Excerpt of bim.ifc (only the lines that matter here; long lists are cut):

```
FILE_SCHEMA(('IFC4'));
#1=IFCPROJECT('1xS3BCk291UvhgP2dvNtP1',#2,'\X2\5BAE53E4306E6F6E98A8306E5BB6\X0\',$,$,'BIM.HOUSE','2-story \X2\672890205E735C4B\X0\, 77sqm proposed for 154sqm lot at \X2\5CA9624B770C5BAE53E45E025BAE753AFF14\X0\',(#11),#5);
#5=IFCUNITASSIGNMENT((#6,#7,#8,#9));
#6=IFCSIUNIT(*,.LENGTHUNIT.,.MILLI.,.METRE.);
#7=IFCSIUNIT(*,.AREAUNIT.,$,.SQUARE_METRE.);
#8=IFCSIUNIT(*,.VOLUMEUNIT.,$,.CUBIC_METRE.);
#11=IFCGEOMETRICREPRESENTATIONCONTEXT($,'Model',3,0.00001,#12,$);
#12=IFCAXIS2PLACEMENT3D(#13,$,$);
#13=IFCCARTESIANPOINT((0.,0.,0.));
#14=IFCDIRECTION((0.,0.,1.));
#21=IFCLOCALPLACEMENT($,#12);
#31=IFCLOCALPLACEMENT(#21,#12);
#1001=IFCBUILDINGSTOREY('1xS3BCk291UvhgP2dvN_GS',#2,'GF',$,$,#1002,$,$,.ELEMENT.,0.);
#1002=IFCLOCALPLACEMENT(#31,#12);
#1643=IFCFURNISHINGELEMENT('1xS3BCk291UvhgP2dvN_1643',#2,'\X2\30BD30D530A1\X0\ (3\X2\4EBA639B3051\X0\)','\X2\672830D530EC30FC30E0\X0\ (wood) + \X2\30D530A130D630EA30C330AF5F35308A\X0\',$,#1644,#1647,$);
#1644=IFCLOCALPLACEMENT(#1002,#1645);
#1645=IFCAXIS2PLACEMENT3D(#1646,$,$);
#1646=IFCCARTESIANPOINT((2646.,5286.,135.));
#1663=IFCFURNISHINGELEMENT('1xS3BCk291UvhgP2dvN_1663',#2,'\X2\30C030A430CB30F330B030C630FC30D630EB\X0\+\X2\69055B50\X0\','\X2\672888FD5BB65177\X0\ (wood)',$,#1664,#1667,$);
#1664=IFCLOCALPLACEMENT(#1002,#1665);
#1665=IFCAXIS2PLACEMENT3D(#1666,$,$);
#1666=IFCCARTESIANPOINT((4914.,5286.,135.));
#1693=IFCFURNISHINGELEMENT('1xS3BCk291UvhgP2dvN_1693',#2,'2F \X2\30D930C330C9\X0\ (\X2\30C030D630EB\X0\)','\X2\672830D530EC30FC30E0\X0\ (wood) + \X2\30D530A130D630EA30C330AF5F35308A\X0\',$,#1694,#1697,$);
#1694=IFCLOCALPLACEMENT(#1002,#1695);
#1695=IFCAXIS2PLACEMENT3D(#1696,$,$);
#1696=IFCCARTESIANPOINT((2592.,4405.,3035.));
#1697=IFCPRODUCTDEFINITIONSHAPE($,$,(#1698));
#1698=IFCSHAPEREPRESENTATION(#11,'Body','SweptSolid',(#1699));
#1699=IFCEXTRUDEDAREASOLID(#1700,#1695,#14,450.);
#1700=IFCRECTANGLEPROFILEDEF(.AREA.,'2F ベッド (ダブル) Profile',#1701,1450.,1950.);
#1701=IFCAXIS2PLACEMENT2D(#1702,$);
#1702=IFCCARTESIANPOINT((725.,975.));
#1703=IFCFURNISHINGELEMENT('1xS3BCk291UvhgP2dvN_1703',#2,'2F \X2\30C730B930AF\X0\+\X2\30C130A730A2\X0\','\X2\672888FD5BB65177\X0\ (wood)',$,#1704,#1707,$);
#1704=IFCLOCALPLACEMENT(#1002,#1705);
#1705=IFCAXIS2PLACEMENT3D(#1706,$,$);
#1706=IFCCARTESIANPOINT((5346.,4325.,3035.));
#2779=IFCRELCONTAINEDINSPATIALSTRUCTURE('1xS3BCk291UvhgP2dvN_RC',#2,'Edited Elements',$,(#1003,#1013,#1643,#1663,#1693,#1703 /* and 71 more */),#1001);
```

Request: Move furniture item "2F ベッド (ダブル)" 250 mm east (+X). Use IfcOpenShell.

```python
import ifcopenshell
import ifcopenshell.api.geometry
import ifcopenshell.util.placement

model = ifcopenshell.open("bim.ifc")

item = model.by_guid("1xS3BCk291UvhgP2dvN_1693")
matrix = ifcopenshell.util.placement.get_local_placement(item.ObjectPlacement)
matrix[0, 3] += 250.0
ifcopenshell.api.geometry.edit_object_placement(model, product=item, matrix=matrix, is_si=False)

print(ifcopenshell.util.placement.get_local_placement(item.ObjectPlacement).round(3) + 0.0)

model.write("bim_rev.ifc")
```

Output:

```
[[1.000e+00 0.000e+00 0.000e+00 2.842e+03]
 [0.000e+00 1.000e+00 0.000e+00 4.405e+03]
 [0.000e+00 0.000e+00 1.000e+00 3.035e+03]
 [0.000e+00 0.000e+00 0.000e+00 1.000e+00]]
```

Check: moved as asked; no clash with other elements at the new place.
